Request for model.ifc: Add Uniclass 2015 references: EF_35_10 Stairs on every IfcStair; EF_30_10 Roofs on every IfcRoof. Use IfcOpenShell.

First a look at what the model holds.

```python
import ifcopenshell

model = ifcopenshell.open("model.ifc")
print(model.schema)
print("classifications:", [c.Name for c in model.by_type("IfcClassification")])
for ifc_class in ("IfcDoor", "IfcRoof", "IfcStair", "IfcWall", "IfcWindow"):
    print(ifc_class, len(model.by_type(ifc_class)))
```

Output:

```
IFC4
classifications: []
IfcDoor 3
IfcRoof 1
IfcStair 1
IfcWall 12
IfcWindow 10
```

```python
import ifcopenshell
import ifcopenshell.api.classification

model = ifcopenshell.open("model.ifc")

system = ifcopenshell.api.classification.add_classification(model, classification="Uniclass 2015")

codes = {
    "IfcStair": ("EF_35_10", "Stairs"),
    "IfcRoof": ("EF_30_10", "Roofs"),
}
for ifc_class, (code, name) in codes.items():
    products = model.by_type(ifc_class)
    ifcopenshell.api.classification.add_reference(
        model, products=products, classification=system, identification=code, name=name
    )
    print(code, len(products))

model.write("model-out.ifc")
```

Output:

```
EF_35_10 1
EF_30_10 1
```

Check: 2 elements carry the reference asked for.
